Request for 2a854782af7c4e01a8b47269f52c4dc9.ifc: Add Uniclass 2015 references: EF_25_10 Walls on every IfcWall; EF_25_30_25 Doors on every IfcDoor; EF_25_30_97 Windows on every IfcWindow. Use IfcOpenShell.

First a look at what the model holds.

```python
import ifcopenshell

model = ifcopenshell.open("2a854782af7c4e01a8b47269f52c4dc9.ifc")
print(model.schema)
print("classifications:", [c.Name for c in model.by_type("IfcClassification")])
for ifc_class in ("IfcDoor", "IfcRoof", "IfcStair", "IfcWall", "IfcWindow"):
    print(ifc_class, len(model.by_type(ifc_class)))
```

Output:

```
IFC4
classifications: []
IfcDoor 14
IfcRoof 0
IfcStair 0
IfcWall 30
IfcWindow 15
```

```python
import ifcopenshell
import ifcopenshell.api.classification

model = ifcopenshell.open("2a854782af7c4e01a8b47269f52c4dc9.ifc")

system = ifcopenshell.api.classification.add_classification(model, classification="Uniclass 2015")

codes = {
    "IfcWall": ("EF_25_10", "Walls"),
    "IfcDoor": ("EF_25_30_25", "Doors"),
    "IfcWindow": ("EF_25_30_97", "Windows"),
}
for ifc_class, (code, name) in codes.items():
    products = model.by_type(ifc_class)
    ifcopenshell.api.classification.add_reference(
        model, products=products, classification=system, identification=code, name=name
    )
    print(code, len(products))

model.write("2a854782af7c4e01a8b47269f52c4dc9_updated.ifc")
```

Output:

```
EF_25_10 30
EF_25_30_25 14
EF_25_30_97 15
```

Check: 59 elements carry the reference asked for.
